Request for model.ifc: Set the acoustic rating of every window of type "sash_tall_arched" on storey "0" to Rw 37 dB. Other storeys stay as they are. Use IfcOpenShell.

First a look at what the model holds.

```python
import ifcopenshell
import ifcopenshell.util.element

model = ifcopenshell.open("model.ifc")
print(model.schema)
storey = next(s for s in model.by_type("IfcBuildingStorey") if s.Name == "0")
windows = [e for e in ifcopenshell.util.element.get_decomposition(storey) if e.is_a("IfcWindow")]
seen = {}
for e in windows:
    element_type = ifcopenshell.util.element.get_type(e)
    key = (element_type.Name if element_type != e and element_type else None, ifcopenshell.util.element.get_pset(e, "Pset_WindowCommon", "AcousticRating"))
    seen[key] = seen.get(key, 0) + 1
for (name, value), count in sorted(seen.items(), key=str):
    print(count, "x", name, "|", value)
```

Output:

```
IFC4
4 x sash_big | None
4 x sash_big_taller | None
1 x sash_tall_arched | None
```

```python
import ifcopenshell
import ifcopenshell.api.pset
import ifcopenshell.util.element

model = ifcopenshell.open("model.ifc")

storey = next(s for s in model.by_type("IfcBuildingStorey") if s.Name == "0")
windows = [e for e in ifcopenshell.util.element.get_decomposition(storey) if e.is_a("IfcWindow")]

count = 0
for e in windows:
    element_type = ifcopenshell.util.element.get_type(e)
    if element_type in (None, e) or element_type.Name != "sash_tall_arched":
        continue
    # add_pset returns the element's existing set when there is one.
    pset = ifcopenshell.api.pset.add_pset(model, product=e, name="Pset_WindowCommon")
    ifcopenshell.api.pset.edit_pset(model, pset=pset, properties={"AcousticRating": "Rw 37 dB"})
    count += 1

print(count, "windows updated")

model.write("model_updated.ifc")
```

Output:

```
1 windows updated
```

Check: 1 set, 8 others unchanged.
